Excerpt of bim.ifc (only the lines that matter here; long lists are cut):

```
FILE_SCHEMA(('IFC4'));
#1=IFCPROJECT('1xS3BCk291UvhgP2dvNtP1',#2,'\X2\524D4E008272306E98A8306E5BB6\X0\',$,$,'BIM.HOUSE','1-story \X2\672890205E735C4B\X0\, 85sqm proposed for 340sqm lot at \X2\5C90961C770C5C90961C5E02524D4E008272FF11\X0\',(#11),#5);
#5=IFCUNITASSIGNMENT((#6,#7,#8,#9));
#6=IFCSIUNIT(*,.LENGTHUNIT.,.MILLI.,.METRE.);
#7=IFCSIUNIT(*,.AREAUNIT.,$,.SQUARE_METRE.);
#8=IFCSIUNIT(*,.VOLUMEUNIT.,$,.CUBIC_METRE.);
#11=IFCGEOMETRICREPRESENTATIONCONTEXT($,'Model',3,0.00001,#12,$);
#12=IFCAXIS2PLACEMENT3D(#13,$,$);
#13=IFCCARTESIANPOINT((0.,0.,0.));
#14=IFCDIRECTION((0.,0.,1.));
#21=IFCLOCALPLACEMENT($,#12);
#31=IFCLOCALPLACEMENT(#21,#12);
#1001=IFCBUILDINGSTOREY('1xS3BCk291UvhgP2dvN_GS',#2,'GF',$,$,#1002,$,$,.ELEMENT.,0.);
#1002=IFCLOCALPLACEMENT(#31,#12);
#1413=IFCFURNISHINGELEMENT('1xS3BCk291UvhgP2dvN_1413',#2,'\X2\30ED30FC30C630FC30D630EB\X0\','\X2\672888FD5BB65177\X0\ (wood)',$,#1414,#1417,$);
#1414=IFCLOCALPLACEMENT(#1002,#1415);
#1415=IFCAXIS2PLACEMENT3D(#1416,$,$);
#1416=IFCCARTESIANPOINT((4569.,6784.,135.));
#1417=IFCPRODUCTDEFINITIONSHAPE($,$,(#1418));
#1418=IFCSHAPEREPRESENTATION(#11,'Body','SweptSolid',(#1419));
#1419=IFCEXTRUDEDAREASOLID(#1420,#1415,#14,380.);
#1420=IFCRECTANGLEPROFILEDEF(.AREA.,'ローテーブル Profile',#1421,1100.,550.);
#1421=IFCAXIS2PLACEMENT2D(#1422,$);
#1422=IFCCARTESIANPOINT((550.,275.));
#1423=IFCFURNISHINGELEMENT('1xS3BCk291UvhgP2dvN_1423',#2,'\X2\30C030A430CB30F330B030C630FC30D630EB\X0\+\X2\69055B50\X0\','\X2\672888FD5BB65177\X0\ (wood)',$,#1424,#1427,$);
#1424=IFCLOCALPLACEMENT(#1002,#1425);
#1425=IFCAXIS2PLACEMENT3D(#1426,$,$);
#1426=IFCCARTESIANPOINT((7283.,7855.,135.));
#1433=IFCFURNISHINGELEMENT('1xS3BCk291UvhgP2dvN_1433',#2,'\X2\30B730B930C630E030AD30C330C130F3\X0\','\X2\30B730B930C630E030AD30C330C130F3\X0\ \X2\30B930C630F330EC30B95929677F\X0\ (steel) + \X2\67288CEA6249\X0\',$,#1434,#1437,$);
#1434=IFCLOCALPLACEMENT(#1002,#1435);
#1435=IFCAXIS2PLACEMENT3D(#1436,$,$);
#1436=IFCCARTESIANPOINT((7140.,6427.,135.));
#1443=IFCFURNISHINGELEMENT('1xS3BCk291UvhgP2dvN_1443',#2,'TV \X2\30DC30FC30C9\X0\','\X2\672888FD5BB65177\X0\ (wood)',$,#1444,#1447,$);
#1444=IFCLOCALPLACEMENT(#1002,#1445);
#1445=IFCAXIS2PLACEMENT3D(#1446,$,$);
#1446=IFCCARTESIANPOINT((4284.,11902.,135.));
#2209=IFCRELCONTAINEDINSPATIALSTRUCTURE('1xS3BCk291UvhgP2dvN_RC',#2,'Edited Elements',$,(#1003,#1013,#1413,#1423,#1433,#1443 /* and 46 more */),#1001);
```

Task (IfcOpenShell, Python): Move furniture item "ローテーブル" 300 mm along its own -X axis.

```python
import ifcopenshell
import ifcopenshell.api.geometry
import ifcopenshell.util.placement
import ifcopenshell.util.unit

model = ifcopenshell.open("bim.ifc")
unit_scale = ifcopenshell.util.unit.calculate_unit_scale(model)

item = model.by_guid("1xS3BCk291UvhgP2dvN_1413")
matrix = ifcopenshell.util.placement.get_local_placement(item.ObjectPlacement)
matrix[:3, 3] -= matrix[:3, 0] * 0.3 / unit_scale
ifcopenshell.api.geometry.edit_object_placement(model, product=item, matrix=matrix, is_si=False)

print(ifcopenshell.util.placement.get_local_placement(item.ObjectPlacement).round(3) + 0.0)

model.write("bim-out.ifc")
```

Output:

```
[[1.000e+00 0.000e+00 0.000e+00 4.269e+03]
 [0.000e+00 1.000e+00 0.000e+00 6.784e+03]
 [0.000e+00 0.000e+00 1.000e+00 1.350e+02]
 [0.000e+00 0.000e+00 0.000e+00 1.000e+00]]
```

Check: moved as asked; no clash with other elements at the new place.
